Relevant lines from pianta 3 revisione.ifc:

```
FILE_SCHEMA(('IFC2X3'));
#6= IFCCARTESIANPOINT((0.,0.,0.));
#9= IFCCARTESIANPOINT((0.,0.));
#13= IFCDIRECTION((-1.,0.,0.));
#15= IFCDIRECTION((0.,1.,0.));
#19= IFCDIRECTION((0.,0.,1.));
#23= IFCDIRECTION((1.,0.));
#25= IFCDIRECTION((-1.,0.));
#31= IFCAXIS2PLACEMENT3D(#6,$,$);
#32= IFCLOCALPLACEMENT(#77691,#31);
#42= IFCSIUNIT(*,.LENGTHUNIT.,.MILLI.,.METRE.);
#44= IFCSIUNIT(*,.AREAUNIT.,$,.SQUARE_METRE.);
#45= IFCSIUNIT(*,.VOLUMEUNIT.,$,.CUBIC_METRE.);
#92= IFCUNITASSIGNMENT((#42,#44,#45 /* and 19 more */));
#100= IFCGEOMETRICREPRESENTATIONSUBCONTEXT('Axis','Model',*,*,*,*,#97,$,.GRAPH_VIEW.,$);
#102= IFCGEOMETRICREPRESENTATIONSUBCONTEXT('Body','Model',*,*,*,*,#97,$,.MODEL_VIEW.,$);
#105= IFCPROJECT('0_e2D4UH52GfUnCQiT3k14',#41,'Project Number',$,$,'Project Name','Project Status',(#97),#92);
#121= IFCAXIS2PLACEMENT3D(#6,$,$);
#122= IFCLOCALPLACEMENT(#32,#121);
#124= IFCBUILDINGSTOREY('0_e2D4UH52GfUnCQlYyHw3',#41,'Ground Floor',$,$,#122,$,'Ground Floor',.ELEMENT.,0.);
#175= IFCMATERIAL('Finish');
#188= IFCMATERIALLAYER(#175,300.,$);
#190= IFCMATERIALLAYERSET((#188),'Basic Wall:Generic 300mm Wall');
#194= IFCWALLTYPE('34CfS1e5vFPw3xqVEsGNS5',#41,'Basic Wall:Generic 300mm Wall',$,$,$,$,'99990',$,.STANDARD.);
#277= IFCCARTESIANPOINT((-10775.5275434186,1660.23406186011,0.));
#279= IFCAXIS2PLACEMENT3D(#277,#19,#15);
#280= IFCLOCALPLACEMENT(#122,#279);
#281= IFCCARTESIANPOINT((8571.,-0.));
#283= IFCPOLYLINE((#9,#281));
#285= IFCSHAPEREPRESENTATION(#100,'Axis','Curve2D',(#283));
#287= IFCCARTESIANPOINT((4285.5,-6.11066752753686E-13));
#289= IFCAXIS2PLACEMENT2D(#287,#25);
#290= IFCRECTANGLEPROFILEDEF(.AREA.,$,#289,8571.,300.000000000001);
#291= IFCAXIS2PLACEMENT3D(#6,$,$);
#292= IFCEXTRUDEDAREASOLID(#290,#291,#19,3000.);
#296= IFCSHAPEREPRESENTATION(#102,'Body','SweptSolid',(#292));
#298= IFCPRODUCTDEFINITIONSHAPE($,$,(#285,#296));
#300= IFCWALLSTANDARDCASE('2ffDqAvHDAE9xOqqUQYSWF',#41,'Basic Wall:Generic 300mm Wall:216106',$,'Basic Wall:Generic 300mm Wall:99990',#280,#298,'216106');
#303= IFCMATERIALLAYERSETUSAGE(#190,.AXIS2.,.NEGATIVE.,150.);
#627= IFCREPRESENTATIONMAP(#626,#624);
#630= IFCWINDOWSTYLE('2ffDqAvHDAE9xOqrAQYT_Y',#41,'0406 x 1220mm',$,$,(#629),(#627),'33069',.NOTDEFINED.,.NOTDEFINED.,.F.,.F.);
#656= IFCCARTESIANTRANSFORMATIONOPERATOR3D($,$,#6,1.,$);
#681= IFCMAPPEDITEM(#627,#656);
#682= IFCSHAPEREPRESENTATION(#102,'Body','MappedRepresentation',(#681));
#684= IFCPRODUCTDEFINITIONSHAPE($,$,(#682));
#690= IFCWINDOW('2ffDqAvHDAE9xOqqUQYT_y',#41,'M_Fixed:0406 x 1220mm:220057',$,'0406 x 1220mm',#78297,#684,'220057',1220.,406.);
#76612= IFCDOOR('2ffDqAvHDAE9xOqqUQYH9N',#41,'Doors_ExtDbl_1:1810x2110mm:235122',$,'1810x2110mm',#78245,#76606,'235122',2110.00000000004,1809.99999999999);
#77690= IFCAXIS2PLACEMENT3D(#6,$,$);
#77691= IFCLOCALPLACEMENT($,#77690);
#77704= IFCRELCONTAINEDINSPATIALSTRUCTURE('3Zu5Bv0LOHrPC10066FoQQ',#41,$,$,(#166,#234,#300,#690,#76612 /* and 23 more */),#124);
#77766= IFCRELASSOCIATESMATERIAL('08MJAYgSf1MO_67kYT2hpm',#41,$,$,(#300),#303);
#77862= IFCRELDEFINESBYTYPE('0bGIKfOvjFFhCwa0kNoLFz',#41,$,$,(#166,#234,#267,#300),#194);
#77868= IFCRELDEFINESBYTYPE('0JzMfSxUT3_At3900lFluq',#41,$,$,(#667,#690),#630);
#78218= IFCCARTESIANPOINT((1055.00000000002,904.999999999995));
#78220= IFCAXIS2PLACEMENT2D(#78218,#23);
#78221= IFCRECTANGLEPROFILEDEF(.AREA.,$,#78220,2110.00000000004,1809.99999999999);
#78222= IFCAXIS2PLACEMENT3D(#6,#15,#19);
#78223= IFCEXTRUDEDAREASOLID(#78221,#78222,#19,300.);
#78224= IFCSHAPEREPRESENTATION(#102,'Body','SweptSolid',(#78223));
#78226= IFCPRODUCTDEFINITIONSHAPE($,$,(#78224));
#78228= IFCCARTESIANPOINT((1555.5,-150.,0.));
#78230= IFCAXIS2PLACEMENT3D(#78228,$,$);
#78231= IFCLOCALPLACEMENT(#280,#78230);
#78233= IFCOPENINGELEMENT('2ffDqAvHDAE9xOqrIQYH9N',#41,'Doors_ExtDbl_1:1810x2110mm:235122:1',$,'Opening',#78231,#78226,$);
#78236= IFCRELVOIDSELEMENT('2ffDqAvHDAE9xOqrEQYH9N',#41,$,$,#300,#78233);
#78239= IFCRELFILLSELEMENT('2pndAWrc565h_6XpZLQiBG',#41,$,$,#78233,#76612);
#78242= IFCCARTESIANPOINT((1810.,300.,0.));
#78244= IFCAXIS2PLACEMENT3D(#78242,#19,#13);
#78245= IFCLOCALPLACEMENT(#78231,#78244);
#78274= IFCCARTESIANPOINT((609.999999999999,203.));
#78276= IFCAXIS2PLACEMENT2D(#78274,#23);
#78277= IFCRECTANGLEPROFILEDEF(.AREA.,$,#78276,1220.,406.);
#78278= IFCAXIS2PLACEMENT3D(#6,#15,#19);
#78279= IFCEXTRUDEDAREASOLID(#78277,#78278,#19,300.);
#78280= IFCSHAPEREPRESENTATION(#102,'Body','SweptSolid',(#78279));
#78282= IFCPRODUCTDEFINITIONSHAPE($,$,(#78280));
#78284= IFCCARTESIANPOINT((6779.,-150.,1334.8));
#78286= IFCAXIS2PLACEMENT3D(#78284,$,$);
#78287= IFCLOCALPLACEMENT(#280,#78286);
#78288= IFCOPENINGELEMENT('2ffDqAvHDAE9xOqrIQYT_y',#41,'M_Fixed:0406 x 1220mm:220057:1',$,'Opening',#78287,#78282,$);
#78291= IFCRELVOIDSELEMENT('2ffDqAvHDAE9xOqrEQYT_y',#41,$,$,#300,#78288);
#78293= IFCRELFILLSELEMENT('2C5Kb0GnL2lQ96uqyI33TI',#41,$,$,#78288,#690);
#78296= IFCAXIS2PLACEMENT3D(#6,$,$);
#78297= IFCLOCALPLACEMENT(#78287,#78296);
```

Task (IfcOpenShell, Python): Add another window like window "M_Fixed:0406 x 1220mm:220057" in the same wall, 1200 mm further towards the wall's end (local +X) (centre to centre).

```python
import ifcopenshell
import ifcopenshell.api.feature
import ifcopenshell.api.geometry
import ifcopenshell.api.root
import ifcopenshell.geom
import ifcopenshell.util.element
import ifcopenshell.util.placement
import ifcopenshell.util.shape
import ifcopenshell.util.unit

model = ifcopenshell.open("pianta 3 revisione.ifc")
unit_scale = ifcopenshell.util.unit.calculate_unit_scale(model)
settings = ifcopenshell.geom.settings()


def volume(element):
    """Net volume in cubic metres, openings subtracted."""
    shape = ifcopenshell.geom.create_shape(settings, element)
    return ifcopenshell.util.shape.get_volume(shape.geometry)


def reuse_history(source, copy):
    """copy_class also copies each property set's owner history, people and application; keep the originals."""
    for rel in copy.IsDefinedBy:
        if rel.is_a("IfcRelDefinesByProperties") and (history := rel.RelatingPropertyDefinition.OwnerHistory):
            rel.RelatingPropertyDefinition.OwnerHistory = source.OwnerHistory
            ifcopenshell.util.element.remove_deep2(model, history)


window = model.by_id(690)
opening = window.FillsVoids[0].RelatingOpeningElement
wall = opening.VoidsElements[0].RelatingBuildingElement
before = volume(wall)
shift = ifcopenshell.util.placement.get_local_placement(wall.ObjectPlacement)[:3, 0] * 1.2 / unit_scale

# copy_class copies the void relationship, type, container and properties, but no geometry.
new_opening = ifcopenshell.api.root.copy_class(model, product=opening)
new_opening.Representation = ifcopenshell.util.element.copy_deep(
    model, opening.Representation, exclude=["IfcGeometricRepresentationContext", "IfcRepresentationMap"]
)
new_opening.Name = "M_Fixed:0406 x 1220mm"
new_window = ifcopenshell.api.root.copy_class(model, product=window)
new_window.Representation = ifcopenshell.util.element.copy_deep(
    model, window.Representation, exclude=["IfcGeometricRepresentationContext", "IfcRepresentationMap"]
)
new_window.Name = "M_Fixed:0406 x 1220mm"
new_window.Tag = None
reuse_history(window, new_window)
fills = ifcopenshell.api.feature.add_filling(model, opening=new_opening, element=new_window)
fills.OwnerHistory = new_window.OwnerHistory  # required in IFC2X3

for old, new in ((opening, new_opening), (window, new_window)):
    matrix = ifcopenshell.util.placement.get_local_placement(old.ObjectPlacement)
    matrix[:3, 3] += shift
    ifcopenshell.api.geometry.edit_object_placement(model, product=new, matrix=matrix, is_si=False)

after = volume(wall)

print(f"wall volume {before:.3f} -> {after:.3f} m3")

model.write("pianta 3 revisione_v2.ifc")
```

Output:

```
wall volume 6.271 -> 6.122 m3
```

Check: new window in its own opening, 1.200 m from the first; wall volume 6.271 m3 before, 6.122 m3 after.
